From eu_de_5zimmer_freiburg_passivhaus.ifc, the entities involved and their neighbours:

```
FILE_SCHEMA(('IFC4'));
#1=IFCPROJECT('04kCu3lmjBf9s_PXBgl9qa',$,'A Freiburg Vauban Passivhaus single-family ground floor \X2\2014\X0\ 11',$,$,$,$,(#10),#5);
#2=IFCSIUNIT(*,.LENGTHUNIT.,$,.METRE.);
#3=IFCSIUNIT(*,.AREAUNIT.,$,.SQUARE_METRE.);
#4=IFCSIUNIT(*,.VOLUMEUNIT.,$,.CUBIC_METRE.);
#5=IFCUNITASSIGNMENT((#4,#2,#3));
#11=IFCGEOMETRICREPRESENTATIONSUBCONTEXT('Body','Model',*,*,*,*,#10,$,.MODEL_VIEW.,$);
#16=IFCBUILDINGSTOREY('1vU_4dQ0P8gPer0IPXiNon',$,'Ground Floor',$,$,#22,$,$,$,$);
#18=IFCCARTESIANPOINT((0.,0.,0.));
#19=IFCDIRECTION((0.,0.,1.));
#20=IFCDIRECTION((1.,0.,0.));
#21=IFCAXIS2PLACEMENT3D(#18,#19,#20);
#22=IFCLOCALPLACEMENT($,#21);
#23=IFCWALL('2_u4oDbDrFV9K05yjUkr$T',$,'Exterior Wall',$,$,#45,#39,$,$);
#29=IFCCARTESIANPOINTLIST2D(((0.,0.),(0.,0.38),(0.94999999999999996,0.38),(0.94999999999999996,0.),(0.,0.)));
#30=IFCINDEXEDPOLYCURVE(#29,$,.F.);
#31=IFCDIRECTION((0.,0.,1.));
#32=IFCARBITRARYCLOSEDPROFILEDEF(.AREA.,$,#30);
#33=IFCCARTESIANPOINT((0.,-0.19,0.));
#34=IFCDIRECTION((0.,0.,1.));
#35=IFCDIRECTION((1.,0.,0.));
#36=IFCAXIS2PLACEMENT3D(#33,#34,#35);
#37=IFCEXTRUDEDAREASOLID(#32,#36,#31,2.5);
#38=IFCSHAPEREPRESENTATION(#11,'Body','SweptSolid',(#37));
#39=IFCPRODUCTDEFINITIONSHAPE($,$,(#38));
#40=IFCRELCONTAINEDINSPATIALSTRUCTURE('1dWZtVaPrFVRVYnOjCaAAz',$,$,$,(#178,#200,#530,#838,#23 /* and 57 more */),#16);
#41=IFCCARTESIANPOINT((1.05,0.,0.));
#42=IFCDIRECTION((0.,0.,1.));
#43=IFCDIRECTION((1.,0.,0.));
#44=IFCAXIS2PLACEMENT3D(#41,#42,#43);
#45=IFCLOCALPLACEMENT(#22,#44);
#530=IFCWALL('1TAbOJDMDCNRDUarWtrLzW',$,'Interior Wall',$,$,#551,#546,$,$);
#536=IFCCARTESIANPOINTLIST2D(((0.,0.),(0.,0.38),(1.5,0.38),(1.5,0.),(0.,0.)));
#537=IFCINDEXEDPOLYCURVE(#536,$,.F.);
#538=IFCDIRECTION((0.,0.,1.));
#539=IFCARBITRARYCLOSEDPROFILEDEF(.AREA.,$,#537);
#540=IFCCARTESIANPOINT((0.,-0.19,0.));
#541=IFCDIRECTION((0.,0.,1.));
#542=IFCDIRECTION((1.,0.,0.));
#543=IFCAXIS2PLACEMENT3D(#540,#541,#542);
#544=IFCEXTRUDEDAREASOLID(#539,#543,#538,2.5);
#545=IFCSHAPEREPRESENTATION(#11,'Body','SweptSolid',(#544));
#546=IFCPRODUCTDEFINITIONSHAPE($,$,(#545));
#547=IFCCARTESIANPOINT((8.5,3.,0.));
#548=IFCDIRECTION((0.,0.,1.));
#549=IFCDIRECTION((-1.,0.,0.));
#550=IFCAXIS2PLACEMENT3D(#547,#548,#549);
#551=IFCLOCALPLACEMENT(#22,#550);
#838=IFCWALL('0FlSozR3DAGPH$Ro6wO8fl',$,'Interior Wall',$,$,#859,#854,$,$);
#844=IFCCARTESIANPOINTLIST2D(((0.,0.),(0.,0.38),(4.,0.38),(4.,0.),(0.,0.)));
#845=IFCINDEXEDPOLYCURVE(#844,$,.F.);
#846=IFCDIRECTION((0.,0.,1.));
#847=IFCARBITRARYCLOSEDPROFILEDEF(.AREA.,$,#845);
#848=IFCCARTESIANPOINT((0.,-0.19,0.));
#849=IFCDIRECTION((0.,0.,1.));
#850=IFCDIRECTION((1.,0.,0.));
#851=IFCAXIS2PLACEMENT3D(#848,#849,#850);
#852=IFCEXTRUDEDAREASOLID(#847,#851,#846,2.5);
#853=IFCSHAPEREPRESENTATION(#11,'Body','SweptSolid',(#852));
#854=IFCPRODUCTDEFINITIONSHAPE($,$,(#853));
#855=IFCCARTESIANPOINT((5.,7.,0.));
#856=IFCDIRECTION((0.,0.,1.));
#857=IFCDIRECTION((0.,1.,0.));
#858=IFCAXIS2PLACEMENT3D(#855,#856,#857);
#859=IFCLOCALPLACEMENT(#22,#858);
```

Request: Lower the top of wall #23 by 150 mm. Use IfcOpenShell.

```python
import ifcopenshell
import ifcopenshell.geom
import ifcopenshell.util.representation
import ifcopenshell.util.shape
import ifcopenshell.util.unit

model = ifcopenshell.open("eu_de_5zimmer_freiburg_passivhaus.ifc")
unit_scale = ifcopenshell.util.unit.calculate_unit_scale(model)
settings = ifcopenshell.geom.settings()


def volume(element):
    """Net volume in cubic metres, openings subtracted."""
    shape = ifcopenshell.geom.create_shape(settings, element)
    return ifcopenshell.util.shape.get_volume(shape.geometry)


wall = model.by_id(23)
before = volume(wall)

body = ifcopenshell.util.representation.get_representation(wall, "Model", "Body")
solid = body.Items[0]
old_height = solid.Depth
solid.Depth -= 0.15 / unit_scale
after = volume(wall)

print(f"height {old_height:g} -> {solid.Depth:g}, volume {before:.3f} -> {after:.3f} m3")

model.write("eu_de_5zimmer_freiburg_passivhaus_rev.ifc")
```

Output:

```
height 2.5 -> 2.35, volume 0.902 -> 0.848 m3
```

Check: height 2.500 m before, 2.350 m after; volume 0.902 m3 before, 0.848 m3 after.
